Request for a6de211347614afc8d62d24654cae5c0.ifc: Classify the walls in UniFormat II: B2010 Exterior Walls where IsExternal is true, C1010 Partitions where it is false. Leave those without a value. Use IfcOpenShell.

First a look at what the model holds.

```python
import ifcopenshell
import ifcopenshell.util.element

model = ifcopenshell.open("a6de211347614afc8d62d24654cae5c0.ifc")
print(model.schema)
print("classifications:", [c.Name for c in model.by_type("IfcClassification")])
values = [ifcopenshell.util.element.get_pset(e, "Pset_WallCommon", "IsExternal") for e in model.by_type("IfcWall")]
for value in (True, False, None):
    print("IsExternal", value, values.count(value))
```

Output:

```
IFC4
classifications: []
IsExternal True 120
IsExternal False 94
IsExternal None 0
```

```python
import ifcopenshell
import ifcopenshell.api.classification
import ifcopenshell.util.element

model = ifcopenshell.open("a6de211347614afc8d62d24654cae5c0.ifc")

system = ifcopenshell.api.classification.add_classification(model, classification="UniFormat II")

walls = model.by_type("IfcWall")
external = {e: ifcopenshell.util.element.get_pset(e, "Pset_WallCommon", "IsExternal") for e in walls}
for flag, code, name in ((True, "B2010", "Exterior Walls"), (False, "C1010", "Partitions")):
    products = [e for e in walls if external[e] is flag]
    ifcopenshell.api.classification.add_reference(
        model, products=products, classification=system, identification=code, name=name
    )
    print(code, len(products))

model.write("a6de211347614afc8d62d24654cae5c0_v2.ifc")
```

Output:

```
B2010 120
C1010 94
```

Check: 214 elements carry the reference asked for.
